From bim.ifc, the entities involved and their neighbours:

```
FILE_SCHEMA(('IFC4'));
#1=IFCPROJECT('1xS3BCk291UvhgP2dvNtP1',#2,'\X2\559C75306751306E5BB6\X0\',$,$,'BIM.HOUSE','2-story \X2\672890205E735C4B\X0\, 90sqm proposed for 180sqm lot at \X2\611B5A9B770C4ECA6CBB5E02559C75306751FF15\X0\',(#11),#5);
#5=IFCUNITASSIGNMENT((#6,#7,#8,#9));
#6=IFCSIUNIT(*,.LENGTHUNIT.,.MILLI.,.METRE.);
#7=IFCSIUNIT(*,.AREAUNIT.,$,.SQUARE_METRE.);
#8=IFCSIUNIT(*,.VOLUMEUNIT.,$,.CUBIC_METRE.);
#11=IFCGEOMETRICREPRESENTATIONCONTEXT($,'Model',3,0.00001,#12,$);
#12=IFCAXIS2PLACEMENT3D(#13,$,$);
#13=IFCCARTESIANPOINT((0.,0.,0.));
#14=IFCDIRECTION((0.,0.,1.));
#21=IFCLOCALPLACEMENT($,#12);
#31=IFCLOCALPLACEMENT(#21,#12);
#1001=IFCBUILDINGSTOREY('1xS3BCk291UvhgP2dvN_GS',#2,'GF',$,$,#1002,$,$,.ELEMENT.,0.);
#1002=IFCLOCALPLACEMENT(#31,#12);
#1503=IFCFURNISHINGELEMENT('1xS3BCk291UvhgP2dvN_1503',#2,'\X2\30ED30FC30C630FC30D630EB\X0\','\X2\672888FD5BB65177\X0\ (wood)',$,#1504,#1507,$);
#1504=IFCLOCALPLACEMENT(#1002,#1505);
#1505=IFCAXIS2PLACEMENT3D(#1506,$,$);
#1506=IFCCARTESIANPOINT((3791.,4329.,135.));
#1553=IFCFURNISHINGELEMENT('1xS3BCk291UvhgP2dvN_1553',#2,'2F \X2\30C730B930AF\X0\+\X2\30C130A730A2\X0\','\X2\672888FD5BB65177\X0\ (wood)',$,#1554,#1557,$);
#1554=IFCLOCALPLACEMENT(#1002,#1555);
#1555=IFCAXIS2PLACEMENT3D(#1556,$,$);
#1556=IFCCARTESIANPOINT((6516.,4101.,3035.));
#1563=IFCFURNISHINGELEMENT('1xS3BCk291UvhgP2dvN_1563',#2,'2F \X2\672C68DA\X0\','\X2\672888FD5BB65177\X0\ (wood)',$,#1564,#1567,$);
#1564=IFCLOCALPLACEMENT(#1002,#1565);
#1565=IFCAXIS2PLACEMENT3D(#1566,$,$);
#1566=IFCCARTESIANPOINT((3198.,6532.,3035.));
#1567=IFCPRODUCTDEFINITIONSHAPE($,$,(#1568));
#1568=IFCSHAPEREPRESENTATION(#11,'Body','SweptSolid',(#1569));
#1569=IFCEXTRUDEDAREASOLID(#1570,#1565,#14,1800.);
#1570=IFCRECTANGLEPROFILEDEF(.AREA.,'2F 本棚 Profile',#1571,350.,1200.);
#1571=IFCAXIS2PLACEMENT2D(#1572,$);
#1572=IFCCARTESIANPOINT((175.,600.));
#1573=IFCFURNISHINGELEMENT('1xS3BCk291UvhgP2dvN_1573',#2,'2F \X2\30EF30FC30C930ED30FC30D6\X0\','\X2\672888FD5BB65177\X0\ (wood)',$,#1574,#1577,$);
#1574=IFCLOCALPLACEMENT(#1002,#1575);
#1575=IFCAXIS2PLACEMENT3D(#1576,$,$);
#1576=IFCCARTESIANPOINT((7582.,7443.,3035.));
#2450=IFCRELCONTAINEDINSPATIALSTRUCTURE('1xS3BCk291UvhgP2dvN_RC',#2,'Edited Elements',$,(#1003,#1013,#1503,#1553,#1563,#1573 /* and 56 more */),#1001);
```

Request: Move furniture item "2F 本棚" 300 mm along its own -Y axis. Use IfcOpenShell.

```python
import ifcopenshell
import ifcopenshell.api.geometry
import ifcopenshell.util.placement
import ifcopenshell.util.unit

model = ifcopenshell.open("bim.ifc")
unit_scale = ifcopenshell.util.unit.calculate_unit_scale(model)

item = model.by_guid("1xS3BCk291UvhgP2dvN_1563")
matrix = ifcopenshell.util.placement.get_local_placement(item.ObjectPlacement)
matrix[:3, 3] -= matrix[:3, 1] * 0.3 / unit_scale
ifcopenshell.api.geometry.edit_object_placement(model, product=item, matrix=matrix, is_si=False)

print(ifcopenshell.util.placement.get_local_placement(item.ObjectPlacement).round(3) + 0.0)

model.write("bim_edited.ifc")
```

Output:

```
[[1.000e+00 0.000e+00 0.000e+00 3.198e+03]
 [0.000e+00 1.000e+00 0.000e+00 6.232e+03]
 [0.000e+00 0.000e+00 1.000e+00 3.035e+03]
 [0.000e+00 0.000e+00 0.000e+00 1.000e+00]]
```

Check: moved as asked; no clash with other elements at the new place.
